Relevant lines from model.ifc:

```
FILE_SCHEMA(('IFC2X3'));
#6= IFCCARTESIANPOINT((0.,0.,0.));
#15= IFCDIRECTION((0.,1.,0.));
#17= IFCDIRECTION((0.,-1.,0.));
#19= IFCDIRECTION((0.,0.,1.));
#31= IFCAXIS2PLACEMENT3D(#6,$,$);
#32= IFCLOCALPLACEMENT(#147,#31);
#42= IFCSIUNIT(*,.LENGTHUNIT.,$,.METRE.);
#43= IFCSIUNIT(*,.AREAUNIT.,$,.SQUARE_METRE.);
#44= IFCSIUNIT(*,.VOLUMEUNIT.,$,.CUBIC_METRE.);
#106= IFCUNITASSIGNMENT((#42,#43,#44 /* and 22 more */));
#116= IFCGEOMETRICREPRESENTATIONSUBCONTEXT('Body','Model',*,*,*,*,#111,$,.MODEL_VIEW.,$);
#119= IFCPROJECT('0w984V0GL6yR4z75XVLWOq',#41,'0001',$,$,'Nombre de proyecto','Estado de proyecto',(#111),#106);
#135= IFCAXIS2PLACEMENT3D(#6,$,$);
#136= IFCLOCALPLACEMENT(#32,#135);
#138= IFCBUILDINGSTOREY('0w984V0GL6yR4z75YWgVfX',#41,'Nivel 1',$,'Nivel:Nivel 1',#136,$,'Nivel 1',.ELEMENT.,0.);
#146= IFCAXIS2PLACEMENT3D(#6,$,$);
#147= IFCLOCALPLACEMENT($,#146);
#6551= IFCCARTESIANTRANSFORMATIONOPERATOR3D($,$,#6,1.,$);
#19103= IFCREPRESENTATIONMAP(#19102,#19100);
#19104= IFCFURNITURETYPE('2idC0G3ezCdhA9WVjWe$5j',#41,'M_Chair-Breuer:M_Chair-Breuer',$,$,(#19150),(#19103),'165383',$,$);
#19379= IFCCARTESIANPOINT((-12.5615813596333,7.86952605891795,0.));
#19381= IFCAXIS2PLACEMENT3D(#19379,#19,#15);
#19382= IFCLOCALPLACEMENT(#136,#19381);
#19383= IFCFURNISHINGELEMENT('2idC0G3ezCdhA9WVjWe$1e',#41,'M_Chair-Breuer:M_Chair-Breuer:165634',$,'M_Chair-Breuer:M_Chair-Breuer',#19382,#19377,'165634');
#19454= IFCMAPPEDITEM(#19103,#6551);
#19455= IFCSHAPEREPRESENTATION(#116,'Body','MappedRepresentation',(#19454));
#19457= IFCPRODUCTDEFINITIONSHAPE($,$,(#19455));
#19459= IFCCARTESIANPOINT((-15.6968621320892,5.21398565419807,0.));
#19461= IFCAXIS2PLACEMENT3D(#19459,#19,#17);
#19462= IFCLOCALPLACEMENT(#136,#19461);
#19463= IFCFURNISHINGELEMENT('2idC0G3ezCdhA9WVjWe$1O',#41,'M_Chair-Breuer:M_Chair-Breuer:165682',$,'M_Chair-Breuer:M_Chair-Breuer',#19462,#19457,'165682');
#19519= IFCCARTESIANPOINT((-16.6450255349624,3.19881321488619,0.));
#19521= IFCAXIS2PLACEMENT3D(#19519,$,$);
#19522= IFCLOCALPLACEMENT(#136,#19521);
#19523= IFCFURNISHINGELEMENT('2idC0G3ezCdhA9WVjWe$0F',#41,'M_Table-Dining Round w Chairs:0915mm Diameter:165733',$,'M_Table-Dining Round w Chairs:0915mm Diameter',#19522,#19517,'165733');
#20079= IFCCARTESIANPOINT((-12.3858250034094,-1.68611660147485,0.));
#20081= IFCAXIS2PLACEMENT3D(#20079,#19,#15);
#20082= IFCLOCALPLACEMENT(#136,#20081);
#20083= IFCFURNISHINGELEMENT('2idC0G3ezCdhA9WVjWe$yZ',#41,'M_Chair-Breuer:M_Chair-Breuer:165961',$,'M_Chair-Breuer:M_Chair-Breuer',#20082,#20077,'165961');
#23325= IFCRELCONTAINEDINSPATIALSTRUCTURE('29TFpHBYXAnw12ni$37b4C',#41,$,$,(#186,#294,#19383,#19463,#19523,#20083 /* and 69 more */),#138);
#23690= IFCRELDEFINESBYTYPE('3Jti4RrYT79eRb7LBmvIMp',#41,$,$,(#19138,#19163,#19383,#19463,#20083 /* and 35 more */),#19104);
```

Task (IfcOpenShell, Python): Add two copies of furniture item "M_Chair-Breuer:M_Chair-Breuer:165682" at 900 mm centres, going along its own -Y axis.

```python
import ifcopenshell
import ifcopenshell.api.geometry
import ifcopenshell.api.root
import ifcopenshell.util.element
import ifcopenshell.util.placement
import ifcopenshell.util.unit

model = ifcopenshell.open("model.ifc")
unit_scale = ifcopenshell.util.unit.calculate_unit_scale(model)


def reuse_history(source, copy):
    """copy_class also copies each property set's owner history, people and application; keep the originals."""
    for rel in copy.IsDefinedBy:
        if rel.is_a("IfcRelDefinesByProperties") and (history := rel.RelatingPropertyDefinition.OwnerHistory):
            rel.RelatingPropertyDefinition.OwnerHistory = source.OwnerHistory
            ifcopenshell.util.element.remove_deep2(model, history)


source = model.by_guid("2idC0G3ezCdhA9WVjWe$1O")
base = ifcopenshell.util.placement.get_local_placement(source.ObjectPlacement)
step = -base[:3, 1] * 0.9 / unit_scale

for i in range(1, 3):
    copy = ifcopenshell.api.root.copy_class(model, product=source)
    copy.Representation = ifcopenshell.util.element.copy_deep(
        model, source.Representation, exclude=["IfcGeometricRepresentationContext", "IfcRepresentationMap"]
    )
    copy.Name = "M_Chair-Breuer:M_Chair-Breuer"
    copy.Tag = None
    reuse_history(source, copy)
    matrix = base.copy()
    matrix[:3, 3] += i * step
    print("added at", matrix[:3, 3].round(3) + 0.0)
    ifcopenshell.api.geometry.edit_object_placement(model, product=copy, matrix=matrix, is_si=False)

model.write("model_rev.ifc")
```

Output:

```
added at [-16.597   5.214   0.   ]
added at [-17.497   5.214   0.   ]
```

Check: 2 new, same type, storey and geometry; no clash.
